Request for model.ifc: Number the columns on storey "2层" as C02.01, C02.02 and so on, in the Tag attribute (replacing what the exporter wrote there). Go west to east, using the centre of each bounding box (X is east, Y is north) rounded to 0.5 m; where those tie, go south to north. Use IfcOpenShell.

First a look at what the model holds.

```python
import ifcopenshell
import ifcopenshell.util.element
import ifcopenshell.util.placement

model = ifcopenshell.open("model.ifc")
print(model.schema)
storey = next(s for s in model.by_type("IfcBuildingStorey") if s.Name == "2层")
columns = [e for e in ifcopenshell.util.element.get_decomposition(storey) if e.is_a("IfcColumn")]
for e in sorted(columns, key=lambda e: e.id()):
    origin = ifcopenshell.util.placement.get_local_placement(e.ObjectPlacement)[:3, 3]
    print(e.id(), e.Tag, e.Name, origin.round(2) + 0.0, sep=" | ")
```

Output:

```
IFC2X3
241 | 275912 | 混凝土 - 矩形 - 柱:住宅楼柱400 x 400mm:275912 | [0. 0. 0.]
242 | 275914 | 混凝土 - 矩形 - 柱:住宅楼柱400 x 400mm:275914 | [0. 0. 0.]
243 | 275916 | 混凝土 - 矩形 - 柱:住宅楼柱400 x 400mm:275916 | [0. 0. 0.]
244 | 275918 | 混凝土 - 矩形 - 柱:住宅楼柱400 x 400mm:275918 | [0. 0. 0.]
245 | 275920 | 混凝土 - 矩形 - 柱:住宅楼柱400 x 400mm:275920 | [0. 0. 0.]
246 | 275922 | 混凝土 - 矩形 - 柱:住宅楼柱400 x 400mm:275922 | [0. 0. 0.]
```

```python
import ifcopenshell
import ifcopenshell.geom
import ifcopenshell.util.element
import ifcopenshell.util.shape

model = ifcopenshell.open("model.ifc")
settings = ifcopenshell.geom.settings()
settings.set("use-world-coords", True)


def centre(element):
    shape = ifcopenshell.geom.create_shape(settings, element)
    return ifcopenshell.util.shape.get_bbox_centroid(shape.geometry)


storey = next(s for s in model.by_type("IfcBuildingStorey") if s.Name == "2层")
columns = [e for e in ifcopenshell.util.element.get_decomposition(storey) if e.is_a("IfcColumn")]

# Insertion points can sit at a corner or the storey origin, so sort by the geometry (in metres).
centres = {e: centre(e) for e in columns}
columns.sort(key=lambda e: (round(centres[e][0] / 0.5), centres[e][1]))

for i, e in enumerate(columns, start=1):
    number = f"C02.{i:02d}"
    e.Tag = number
    print(e.id(), number)

model.write("model_updated.ifc")
```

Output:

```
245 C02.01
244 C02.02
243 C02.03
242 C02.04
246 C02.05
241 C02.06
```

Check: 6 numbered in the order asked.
